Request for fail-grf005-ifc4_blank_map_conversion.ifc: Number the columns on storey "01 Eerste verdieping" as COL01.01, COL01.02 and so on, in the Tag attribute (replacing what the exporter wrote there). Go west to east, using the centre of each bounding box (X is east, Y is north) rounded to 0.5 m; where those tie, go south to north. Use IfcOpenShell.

First a look at what the model holds.

```python
import ifcopenshell
import ifcopenshell.util.element
import ifcopenshell.util.placement

model = ifcopenshell.open("fail-grf005-ifc4_blank_map_conversion.ifc")
print(model.schema)
storey = next(s for s in model.by_type("IfcBuildingStorey") if s.Name == "01 Eerste verdieping")
columns = [e for e in ifcopenshell.util.element.get_decomposition(storey) if e.is_a("IfcColumn")]
for e in sorted(columns, key=lambda e: e.id()):
    origin = ifcopenshell.util.placement.get_local_placement(e.ObjectPlacement)[:3, 3]
    print(e.id(), e.Tag, e.Name, origin.round(2) + 0.0, sep=" | ")
```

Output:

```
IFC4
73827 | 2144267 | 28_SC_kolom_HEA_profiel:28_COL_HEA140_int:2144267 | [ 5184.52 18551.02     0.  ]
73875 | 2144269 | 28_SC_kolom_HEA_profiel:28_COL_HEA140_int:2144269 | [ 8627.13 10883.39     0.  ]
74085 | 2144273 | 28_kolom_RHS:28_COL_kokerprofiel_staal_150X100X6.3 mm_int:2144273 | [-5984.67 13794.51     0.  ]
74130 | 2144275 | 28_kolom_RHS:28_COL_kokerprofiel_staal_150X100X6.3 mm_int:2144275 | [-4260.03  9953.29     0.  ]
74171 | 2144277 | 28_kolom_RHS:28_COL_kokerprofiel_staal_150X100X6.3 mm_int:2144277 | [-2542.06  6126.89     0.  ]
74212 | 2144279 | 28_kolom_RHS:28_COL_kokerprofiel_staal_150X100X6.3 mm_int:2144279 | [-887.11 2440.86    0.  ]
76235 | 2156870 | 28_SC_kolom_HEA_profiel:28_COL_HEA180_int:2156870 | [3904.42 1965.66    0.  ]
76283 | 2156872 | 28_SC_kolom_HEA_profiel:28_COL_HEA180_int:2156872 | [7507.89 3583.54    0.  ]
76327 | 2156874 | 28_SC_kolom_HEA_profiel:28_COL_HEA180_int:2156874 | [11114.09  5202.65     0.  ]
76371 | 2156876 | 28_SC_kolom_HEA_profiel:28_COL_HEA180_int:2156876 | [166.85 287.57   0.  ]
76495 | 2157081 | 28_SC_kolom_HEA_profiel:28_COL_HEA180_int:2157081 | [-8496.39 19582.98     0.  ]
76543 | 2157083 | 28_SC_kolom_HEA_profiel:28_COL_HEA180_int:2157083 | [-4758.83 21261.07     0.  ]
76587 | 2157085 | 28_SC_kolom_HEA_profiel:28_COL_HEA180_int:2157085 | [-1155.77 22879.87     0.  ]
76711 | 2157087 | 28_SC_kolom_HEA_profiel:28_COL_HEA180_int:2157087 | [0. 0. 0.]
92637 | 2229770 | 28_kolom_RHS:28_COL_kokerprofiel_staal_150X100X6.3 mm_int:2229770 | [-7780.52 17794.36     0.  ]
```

```python
import ifcopenshell
import ifcopenshell.geom
import ifcopenshell.util.element
import ifcopenshell.util.shape

model = ifcopenshell.open("fail-grf005-ifc4_blank_map_conversion.ifc")
settings = ifcopenshell.geom.settings()
settings.set("use-world-coords", True)


def centre(element):
    shape = ifcopenshell.geom.create_shape(settings, element)
    return ifcopenshell.util.shape.get_bbox_centroid(shape.geometry)


storey = next(s for s in model.by_type("IfcBuildingStorey") if s.Name == "01 Eerste verdieping")
columns = [e for e in ifcopenshell.util.element.get_decomposition(storey) if e.is_a("IfcColumn")]

# Insertion points can sit at a corner or the storey origin, so sort by the geometry (in metres).
centres = {e: centre(e) for e in columns}
columns.sort(key=lambda e: (round(centres[e][0] / 0.5), centres[e][1]))

for i, e in enumerate(columns, start=1):
    number = f"COL01.{i:02d}"
    e.Tag = number
    print(e.id(), number)

model.write("fail-grf005-ifc4_blank_map_conversion_edited.ifc")
```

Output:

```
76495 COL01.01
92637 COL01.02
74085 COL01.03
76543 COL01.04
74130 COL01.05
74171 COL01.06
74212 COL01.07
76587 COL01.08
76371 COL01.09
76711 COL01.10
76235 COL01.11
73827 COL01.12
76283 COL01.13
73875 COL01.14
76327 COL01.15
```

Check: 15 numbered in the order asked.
